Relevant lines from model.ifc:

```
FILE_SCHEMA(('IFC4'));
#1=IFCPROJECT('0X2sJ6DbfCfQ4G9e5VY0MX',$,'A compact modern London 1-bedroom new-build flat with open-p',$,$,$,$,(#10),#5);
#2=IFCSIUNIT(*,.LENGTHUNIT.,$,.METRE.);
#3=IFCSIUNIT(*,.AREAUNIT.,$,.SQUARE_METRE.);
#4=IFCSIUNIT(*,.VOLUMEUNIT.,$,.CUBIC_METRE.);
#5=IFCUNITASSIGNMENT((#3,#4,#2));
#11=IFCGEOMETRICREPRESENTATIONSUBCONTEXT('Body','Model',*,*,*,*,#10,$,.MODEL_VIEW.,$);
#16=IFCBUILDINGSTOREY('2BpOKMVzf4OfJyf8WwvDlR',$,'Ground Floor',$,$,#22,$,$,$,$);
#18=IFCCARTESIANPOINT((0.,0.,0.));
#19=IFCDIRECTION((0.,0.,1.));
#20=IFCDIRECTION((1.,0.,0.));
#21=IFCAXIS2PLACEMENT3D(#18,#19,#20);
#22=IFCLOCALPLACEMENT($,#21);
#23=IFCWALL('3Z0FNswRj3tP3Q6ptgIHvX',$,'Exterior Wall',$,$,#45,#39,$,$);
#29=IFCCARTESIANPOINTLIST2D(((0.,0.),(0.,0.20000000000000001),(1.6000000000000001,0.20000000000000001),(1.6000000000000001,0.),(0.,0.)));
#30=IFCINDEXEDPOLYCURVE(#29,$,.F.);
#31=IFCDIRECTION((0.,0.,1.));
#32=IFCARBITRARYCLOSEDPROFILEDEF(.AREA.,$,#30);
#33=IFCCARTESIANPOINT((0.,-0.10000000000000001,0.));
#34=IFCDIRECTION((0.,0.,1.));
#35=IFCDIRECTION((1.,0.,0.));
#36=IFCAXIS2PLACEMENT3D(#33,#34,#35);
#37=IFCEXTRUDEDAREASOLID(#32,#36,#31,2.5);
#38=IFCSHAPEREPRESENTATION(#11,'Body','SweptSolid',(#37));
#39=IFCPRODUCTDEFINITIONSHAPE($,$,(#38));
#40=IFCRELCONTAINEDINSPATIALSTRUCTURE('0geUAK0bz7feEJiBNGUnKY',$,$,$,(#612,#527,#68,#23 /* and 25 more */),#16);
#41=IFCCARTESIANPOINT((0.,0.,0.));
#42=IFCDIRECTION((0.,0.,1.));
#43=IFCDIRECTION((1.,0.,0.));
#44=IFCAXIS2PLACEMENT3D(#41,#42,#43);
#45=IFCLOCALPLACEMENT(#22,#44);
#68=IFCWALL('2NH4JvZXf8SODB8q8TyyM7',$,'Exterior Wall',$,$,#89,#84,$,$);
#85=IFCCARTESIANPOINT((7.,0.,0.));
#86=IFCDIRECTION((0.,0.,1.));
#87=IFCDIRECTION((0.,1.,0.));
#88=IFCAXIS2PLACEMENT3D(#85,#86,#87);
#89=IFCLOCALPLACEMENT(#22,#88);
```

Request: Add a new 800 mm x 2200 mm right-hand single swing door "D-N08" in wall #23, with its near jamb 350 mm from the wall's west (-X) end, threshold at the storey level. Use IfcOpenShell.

```python
import numpy as np
import ifcopenshell
import ifcopenshell.api.feature
import ifcopenshell.api.geometry
import ifcopenshell.api.root
import ifcopenshell.api.spatial
import ifcopenshell.geom
import ifcopenshell.util.element
import ifcopenshell.util.placement
import ifcopenshell.util.representation
import ifcopenshell.util.shape
import ifcopenshell.util.unit

model = ifcopenshell.open("model.ifc")
unit_scale = ifcopenshell.util.unit.calculate_unit_scale(model)
settings = ifcopenshell.geom.settings()


def volume(element):
    """Net volume in cubic metres, openings subtracted."""
    shape = ifcopenshell.geom.create_shape(settings, element)
    return ifcopenshell.util.shape.get_volume(shape.geometry)


wall = model.by_guid("3Z0FNswRj3tP3Q6ptgIHvX")
storey = ifcopenshell.util.element.get_container(wall, ifc_class="IfcBuildingStorey")
context = ifcopenshell.util.representation.get_context(model, "Model", "Body", "MODEL_VIEW")
before = volume(wall)

width, height, from_end, sill = 0.8, 2.2, 0.35, 0.0  # metres

# The wall runs along its own X axis, and the end named is its -X end.
wall_shape = ifcopenshell.geom.create_shape(settings, wall)
x, y, z = ifcopenshell.util.shape.get_vertices(wall_shape.geometry).T
start = x.min() + from_end
face, thickness = float(y.min()), float(y.max() - y.min())
wall_matrix = ifcopenshell.util.placement.get_local_placement(wall.ObjectPlacement)
level = ifcopenshell.util.placement.get_local_placement(storey.ObjectPlacement)[2, 3]


def in_wall(x, y):
    """Placement at x, y metres in the wall's axes, at sill height."""
    matrix = wall_matrix.copy()
    matrix[:, 3] = wall_matrix @ np.array([x / unit_scale, y / unit_scale, 0.0, 1.0])
    matrix[2, 3] = level + sill / unit_scale
    return matrix


# Opening: a box that overshoots both wall faces by 50 mm.
opening = ifcopenshell.api.root.create_entity(model, ifc_class="IfcOpeningElement", predefined_type="OPENING")
box = ifcopenshell.api.geometry.add_wall_representation(
    model, context=context, length=width, height=height, thickness=thickness + 0.1
)
ifcopenshell.api.geometry.assign_representation(model, product=opening, representation=box)
ifcopenshell.api.geometry.edit_object_placement(model, product=opening, matrix=in_wall(start, face - 0.05), is_si=False)
ifcopenshell.api.feature.add_feature(model, feature=opening, element=wall)

door = ifcopenshell.api.root.create_entity(model, ifc_class="IfcDoor", name="D-N08", predefined_type="DOOR")
door.OverallWidth, door.OverallHeight = width / unit_scale, height / unit_scale
door.OperationType = "SINGLE_SWING_RIGHT"
body = ifcopenshell.api.geometry.add_door_representation(
    model,
    context=context,
    overall_width=door.OverallWidth,
    overall_height=door.OverallHeight,
    operation_type="SINGLE_SWING_RIGHT",
    lining_properties={"LiningDepth": thickness / unit_scale, "ThresholdDepth": thickness / unit_scale},
)
ifcopenshell.api.geometry.assign_representation(model, product=door, representation=body)
ifcopenshell.api.spatial.assign_container(model, products=[door], relating_structure=storey)
ifcopenshell.api.feature.add_filling(model, opening=opening, element=door)

# The lining spans the wall, so the door starts at the wall face.
ifcopenshell.api.geometry.edit_object_placement(model, product=door, matrix=in_wall(start, face), is_si=False)

after = volume(wall)

print(f"wall volume {before:.3f} -> {after:.3f} m3")

model.write("model_rev.ifc")
```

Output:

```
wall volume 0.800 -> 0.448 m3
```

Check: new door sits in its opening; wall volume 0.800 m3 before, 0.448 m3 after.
